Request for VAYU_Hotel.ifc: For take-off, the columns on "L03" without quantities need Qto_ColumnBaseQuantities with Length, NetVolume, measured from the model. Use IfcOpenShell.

First a look at what the model holds.

```python
import ifcopenshell
import ifcopenshell.util.element
import ifcopenshell.util.unit

model = ifcopenshell.open("VAYU_Hotel.ifc")
print(model.schema)
for unit_type in ("LENGTHUNIT", "AREAUNIT", "VOLUMEUNIT"):
    print(unit_type, ifcopenshell.util.unit.calculate_unit_scale(model, unit_type))
storey = next(s for s in model.by_type("IfcBuildingStorey") if s.Name == "L03")
columns = [e for e in ifcopenshell.util.element.get_decomposition(storey) if e.is_a("IfcColumn")]
for e in sorted(columns, key=lambda e: e.id()):
    print(e.id(), e.is_a(), e.Name, list(ifcopenshell.util.element.get_psets(e, qtos_only=True)), sep=" | ")
```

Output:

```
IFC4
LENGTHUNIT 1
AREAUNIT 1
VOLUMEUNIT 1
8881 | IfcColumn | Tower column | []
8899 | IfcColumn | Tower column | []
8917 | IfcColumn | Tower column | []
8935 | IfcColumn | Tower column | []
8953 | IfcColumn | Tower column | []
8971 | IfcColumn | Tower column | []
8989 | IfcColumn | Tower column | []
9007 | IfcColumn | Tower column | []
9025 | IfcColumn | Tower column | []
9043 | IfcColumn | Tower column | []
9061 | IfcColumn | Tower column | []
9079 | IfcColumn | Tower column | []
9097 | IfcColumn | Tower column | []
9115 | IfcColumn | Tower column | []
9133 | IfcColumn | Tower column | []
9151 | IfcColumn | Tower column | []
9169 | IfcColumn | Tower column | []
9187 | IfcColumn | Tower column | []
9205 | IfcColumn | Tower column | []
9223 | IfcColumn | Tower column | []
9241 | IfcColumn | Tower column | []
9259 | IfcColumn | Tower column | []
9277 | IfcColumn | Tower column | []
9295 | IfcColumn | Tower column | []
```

```python
import ifcopenshell
import ifcopenshell.api.pset
import ifcopenshell.geom
import ifcopenshell.util.element
import ifcopenshell.util.shape
import ifcopenshell.util.unit

model = ifcopenshell.open("VAYU_Hotel.ifc")
unit_scale = ifcopenshell.util.unit.calculate_unit_scale(model)
volume_scale = ifcopenshell.util.unit.calculate_unit_scale(model, "VOLUMEUNIT")
settings = ifcopenshell.geom.settings()

storey = next(s for s in model.by_type("IfcBuildingStorey") if s.Name == "L03")
columns = [e for e in ifcopenshell.util.element.get_decomposition(storey) if e.is_a("IfcColumn")]

for e in sorted(columns, key=lambda e: e.id()):
    if ifcopenshell.util.element.get_psets(e, qtos_only=True, should_inherit=False):
        continue
    # Geometry comes back in metres, in the element's own axes.
    shape = ifcopenshell.geom.create_shape(settings, e)
    values = {
        "Length": ifcopenshell.util.shape.get_z(shape.geometry) / unit_scale,
        "NetVolume": ifcopenshell.util.shape.get_volume(shape.geometry) / volume_scale,
    }
    qto = ifcopenshell.api.pset.add_qto(model, product=e, name="Qto_ColumnBaseQuantities")
    ifcopenshell.api.pset.edit_qto(model, qto=qto, properties=values)
    print(e.id(), {k: round(v, 3) for k, v in values.items()})

model.write("VAYU_Hotel_v2.ifc")
```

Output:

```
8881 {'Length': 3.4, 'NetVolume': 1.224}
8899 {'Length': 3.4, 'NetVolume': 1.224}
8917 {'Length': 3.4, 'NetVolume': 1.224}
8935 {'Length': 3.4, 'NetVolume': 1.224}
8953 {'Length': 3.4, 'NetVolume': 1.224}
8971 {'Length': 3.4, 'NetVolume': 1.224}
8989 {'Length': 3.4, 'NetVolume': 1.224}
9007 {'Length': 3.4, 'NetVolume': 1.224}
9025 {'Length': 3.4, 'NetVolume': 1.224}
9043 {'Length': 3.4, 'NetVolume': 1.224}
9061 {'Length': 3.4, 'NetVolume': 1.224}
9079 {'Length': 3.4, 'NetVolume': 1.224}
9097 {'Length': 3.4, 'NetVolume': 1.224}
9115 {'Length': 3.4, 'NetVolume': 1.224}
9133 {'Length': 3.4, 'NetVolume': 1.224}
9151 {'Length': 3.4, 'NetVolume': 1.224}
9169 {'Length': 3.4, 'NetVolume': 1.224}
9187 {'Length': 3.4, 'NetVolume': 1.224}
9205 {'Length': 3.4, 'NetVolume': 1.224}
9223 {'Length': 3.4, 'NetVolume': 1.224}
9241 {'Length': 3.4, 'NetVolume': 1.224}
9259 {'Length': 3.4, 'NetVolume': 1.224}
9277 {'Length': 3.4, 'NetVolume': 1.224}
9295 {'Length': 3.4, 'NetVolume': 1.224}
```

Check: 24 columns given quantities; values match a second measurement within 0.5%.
